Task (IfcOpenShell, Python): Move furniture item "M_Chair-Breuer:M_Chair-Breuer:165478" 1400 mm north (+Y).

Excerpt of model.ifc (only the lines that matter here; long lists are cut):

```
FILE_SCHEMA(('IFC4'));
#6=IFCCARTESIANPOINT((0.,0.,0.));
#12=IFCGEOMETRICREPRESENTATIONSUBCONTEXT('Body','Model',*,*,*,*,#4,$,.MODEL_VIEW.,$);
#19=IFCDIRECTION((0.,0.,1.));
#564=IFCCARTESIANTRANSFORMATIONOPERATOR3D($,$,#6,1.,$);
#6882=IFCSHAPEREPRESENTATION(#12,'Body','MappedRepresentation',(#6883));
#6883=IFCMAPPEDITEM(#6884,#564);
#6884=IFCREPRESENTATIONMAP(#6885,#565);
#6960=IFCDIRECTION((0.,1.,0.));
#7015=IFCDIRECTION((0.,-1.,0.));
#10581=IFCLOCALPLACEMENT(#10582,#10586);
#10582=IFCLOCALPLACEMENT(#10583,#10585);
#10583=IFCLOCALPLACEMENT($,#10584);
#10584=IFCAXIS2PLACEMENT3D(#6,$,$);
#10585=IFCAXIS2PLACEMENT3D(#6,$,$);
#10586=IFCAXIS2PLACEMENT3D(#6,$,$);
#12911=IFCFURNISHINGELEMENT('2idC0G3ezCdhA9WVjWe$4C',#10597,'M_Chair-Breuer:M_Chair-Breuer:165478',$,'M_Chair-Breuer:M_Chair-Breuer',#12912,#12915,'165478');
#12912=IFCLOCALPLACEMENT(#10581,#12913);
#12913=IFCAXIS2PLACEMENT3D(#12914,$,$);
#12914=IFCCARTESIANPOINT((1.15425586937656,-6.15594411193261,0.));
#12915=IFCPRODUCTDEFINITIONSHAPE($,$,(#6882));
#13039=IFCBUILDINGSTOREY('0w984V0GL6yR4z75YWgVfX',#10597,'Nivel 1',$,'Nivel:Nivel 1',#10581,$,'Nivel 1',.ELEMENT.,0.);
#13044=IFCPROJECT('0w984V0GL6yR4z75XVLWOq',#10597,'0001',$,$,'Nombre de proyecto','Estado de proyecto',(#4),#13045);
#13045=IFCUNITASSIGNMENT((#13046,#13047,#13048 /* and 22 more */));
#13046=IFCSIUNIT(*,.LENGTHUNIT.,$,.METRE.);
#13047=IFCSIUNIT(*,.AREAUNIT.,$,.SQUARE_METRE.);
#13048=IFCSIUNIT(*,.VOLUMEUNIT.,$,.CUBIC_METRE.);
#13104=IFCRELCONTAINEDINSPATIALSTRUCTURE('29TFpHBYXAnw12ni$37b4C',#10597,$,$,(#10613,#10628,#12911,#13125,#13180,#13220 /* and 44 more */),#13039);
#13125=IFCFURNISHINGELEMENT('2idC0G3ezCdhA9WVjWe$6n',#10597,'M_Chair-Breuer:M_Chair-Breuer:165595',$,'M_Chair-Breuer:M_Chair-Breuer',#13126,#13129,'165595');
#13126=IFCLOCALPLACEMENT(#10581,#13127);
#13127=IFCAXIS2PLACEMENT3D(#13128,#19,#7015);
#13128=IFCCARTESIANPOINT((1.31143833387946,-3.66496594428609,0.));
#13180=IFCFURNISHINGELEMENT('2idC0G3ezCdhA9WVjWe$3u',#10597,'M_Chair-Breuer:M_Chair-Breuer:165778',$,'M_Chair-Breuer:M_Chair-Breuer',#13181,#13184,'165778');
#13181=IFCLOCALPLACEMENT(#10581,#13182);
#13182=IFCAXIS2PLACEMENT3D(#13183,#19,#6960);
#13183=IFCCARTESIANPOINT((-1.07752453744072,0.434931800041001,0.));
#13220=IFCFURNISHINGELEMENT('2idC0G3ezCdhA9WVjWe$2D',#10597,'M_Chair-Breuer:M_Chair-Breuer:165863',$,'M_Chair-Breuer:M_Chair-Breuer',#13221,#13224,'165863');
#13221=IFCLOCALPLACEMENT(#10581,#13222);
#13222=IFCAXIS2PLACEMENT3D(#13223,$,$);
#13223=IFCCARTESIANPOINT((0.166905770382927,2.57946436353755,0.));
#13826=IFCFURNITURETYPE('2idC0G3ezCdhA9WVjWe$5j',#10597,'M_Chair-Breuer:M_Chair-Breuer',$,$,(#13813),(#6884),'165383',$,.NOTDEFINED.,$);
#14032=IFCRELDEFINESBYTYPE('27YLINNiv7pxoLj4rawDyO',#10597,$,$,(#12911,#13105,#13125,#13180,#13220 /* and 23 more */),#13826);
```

```python
import ifcopenshell
import ifcopenshell.api.geometry
import ifcopenshell.util.placement

model = ifcopenshell.open("model.ifc")

item = model.by_id(12911)
matrix = ifcopenshell.util.placement.get_local_placement(item.ObjectPlacement)
matrix[1, 3] += 1.4
ifcopenshell.api.geometry.edit_object_placement(model, product=item, matrix=matrix, is_si=False)

print(ifcopenshell.util.placement.get_local_placement(item.ObjectPlacement).round(3) + 0.0)

model.write("model_updated.ifc")
```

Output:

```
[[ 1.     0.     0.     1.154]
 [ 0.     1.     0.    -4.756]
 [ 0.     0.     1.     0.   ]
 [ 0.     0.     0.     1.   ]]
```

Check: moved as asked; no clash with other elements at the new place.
